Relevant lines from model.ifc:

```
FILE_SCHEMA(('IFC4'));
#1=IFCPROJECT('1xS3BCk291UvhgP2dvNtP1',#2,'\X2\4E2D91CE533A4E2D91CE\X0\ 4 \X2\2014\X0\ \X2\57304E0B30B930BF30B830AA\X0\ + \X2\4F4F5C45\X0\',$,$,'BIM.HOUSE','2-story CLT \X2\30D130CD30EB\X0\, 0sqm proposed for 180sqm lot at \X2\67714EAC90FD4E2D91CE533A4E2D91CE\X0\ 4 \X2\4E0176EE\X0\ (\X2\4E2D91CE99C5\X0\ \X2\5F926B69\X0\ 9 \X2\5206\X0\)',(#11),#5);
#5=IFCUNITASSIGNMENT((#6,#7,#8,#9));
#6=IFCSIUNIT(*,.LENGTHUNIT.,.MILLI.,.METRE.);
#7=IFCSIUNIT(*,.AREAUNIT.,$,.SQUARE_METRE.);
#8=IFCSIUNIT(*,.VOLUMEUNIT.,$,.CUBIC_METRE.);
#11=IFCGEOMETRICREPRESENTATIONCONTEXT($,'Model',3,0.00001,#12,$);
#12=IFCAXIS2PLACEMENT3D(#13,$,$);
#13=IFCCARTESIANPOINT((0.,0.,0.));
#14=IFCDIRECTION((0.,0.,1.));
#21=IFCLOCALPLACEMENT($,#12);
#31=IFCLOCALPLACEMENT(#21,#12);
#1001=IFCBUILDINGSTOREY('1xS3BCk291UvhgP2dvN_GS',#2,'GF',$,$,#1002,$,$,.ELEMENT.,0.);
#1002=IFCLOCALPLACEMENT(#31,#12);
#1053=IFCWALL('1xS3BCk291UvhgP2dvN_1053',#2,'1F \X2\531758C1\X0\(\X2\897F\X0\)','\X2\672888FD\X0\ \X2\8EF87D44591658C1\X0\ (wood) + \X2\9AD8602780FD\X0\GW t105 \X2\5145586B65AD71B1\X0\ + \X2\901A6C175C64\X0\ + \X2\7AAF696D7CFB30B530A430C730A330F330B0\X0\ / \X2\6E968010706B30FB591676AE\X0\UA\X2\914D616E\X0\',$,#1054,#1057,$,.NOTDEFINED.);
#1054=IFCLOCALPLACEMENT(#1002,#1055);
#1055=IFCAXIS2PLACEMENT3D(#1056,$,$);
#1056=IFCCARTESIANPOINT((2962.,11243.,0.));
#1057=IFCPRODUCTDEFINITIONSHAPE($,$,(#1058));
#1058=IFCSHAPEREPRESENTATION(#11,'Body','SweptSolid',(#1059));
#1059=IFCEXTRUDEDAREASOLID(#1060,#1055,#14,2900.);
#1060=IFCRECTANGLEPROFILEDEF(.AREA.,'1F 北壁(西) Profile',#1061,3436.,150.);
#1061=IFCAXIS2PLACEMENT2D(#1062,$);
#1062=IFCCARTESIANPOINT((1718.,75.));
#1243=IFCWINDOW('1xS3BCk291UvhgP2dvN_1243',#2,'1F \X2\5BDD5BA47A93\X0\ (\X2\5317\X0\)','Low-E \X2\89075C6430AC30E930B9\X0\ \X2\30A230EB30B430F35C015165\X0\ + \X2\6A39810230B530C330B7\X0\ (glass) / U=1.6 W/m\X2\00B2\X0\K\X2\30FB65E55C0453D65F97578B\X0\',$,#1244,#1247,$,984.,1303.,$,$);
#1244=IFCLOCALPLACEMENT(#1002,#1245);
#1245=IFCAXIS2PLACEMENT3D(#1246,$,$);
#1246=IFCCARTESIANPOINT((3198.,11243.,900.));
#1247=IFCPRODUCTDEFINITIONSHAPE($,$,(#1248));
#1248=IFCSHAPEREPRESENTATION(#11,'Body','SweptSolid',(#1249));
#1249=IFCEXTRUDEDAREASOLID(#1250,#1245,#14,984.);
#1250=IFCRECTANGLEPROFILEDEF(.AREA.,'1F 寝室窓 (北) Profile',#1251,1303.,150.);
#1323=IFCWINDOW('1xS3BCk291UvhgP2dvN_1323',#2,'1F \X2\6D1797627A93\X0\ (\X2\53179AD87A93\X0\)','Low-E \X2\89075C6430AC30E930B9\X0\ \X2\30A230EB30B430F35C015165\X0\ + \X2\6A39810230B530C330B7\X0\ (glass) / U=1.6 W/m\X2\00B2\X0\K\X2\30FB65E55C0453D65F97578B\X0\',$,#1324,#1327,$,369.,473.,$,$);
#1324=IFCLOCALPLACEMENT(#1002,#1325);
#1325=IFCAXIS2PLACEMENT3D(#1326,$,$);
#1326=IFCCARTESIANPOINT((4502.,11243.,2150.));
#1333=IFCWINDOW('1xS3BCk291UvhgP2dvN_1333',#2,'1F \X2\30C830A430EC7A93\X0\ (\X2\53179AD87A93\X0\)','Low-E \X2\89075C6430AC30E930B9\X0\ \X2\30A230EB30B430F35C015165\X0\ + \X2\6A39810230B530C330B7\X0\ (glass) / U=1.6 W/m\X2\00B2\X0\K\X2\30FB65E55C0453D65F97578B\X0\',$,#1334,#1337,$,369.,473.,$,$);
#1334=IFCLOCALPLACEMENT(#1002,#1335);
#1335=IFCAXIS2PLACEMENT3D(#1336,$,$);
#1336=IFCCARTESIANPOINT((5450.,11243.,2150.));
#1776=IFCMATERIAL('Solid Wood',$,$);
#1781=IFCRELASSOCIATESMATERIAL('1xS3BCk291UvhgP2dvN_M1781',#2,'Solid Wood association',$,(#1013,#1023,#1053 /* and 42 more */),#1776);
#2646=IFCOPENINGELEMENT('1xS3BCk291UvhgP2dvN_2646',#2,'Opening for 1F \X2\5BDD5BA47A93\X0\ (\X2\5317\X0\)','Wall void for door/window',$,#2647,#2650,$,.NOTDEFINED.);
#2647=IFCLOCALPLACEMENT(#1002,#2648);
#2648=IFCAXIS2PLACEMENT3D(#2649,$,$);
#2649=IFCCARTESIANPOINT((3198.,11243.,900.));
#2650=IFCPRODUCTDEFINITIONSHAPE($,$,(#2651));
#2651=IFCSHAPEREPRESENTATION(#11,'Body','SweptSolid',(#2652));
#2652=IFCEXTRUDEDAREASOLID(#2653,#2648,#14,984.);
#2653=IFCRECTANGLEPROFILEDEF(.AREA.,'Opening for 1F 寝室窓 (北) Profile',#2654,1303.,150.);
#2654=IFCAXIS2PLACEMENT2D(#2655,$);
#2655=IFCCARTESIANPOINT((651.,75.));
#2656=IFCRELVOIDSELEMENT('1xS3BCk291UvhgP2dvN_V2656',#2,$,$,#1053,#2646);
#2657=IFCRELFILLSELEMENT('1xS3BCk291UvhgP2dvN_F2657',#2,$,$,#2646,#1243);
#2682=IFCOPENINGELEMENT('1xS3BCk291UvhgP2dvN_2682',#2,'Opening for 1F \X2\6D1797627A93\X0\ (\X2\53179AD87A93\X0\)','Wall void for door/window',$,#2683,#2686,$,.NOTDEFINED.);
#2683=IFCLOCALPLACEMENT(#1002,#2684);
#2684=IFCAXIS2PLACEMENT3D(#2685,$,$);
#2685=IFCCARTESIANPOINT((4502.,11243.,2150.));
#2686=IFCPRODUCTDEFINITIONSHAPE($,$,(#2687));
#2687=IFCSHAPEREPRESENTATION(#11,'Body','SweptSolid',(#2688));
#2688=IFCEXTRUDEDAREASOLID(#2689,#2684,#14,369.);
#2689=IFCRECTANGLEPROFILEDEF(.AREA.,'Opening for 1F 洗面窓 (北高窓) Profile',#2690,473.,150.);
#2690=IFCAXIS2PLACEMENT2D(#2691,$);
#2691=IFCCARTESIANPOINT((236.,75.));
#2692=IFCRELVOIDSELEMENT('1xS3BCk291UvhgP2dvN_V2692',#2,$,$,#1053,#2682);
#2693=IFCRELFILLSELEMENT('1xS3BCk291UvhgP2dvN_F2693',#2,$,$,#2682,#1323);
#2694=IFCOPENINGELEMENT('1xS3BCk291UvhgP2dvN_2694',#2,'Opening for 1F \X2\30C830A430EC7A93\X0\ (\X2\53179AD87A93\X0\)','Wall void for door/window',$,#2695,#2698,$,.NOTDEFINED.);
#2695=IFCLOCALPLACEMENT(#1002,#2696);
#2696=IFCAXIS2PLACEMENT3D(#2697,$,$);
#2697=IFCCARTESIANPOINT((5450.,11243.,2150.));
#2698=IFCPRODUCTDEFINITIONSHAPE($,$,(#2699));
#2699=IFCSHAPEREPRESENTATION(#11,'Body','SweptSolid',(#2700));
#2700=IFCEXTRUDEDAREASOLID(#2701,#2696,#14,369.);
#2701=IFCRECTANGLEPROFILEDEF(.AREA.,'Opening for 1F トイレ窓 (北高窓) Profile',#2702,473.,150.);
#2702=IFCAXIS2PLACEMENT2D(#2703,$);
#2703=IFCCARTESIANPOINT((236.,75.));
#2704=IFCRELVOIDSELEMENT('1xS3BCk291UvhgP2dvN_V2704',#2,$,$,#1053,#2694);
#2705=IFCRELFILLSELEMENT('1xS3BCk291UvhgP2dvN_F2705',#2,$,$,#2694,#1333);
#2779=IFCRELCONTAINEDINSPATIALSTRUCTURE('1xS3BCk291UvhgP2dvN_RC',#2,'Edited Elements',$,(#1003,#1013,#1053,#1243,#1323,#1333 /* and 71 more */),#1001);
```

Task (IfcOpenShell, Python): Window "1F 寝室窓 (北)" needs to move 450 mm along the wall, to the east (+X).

```python
import ifcopenshell
import ifcopenshell.api.geometry
import ifcopenshell.util.placement

model = ifcopenshell.open("model.ifc")

window = model.by_guid("1xS3BCk291UvhgP2dvN_1243")
opening = window.FillsVoids[0].RelatingOpeningElement
wall = opening.VoidsElements[0].RelatingBuildingElement

wall_matrix = ifcopenshell.util.placement.get_local_placement(wall.ObjectPlacement)
shift = wall_matrix[:3, 0] * 450.0
before = ifcopenshell.util.placement.get_local_placement(window.ObjectPlacement)[:3, 3].copy()

# The window is not placed relative to its opening, so move both.
for product in (opening, window):
    matrix = ifcopenshell.util.placement.get_local_placement(product.ObjectPlacement)
    matrix[:3, 3] += shift
    ifcopenshell.api.geometry.edit_object_placement(model, product=product, matrix=matrix, is_si=False)

after = ifcopenshell.util.placement.get_local_placement(window.ObjectPlacement)[:3, 3]
print("window moved by", (after - before).round(3) + 0.0)

model.write("model_rev.ifc")
```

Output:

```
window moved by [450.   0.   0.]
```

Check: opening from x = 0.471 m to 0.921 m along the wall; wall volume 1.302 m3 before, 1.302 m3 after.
